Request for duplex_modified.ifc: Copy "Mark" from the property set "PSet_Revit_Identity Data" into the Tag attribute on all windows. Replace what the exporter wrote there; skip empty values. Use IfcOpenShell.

First a look at what the model holds.

```python
import ifcopenshell
import ifcopenshell.util.element

model = ifcopenshell.open("duplex_modified.ifc")
print(model.schema)
windows = model.by_type("IfcWindow")
print(len(windows), "windows")
for e in windows[:8]:
    source = ifcopenshell.util.element.get_pset(e, "PSet_Revit_Identity Data", "Mark")
    target = e.Tag
    print(e.id(), repr(source), repr(target), sep=" | ")
```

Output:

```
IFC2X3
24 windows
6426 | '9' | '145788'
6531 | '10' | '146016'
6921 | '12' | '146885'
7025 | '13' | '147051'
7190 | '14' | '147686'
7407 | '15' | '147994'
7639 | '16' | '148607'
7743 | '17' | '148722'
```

```python
import ifcopenshell
import ifcopenshell.util.element

model = ifcopenshell.open("duplex_modified.ifc")

count = 0
for e in model.by_type("IfcWindow"):
    value = ifcopenshell.util.element.get_pset(e, "PSet_Revit_Identity Data", "Mark")
    current = e.Tag
    if not value or not value.strip() or current == value:
        continue
    e.Tag = value
    count += 1

print(count, "windows updated")

model.write("duplex_modified_edited.ifc")
```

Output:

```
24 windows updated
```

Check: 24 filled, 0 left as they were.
